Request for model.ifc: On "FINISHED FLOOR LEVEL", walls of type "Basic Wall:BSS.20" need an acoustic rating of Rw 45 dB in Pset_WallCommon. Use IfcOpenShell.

First a look at what the model holds.

```python
import ifcopenshell
import ifcopenshell.util.element

model = ifcopenshell.open("model.ifc")
print(model.schema)
storey = next(s for s in model.by_type("IfcBuildingStorey") if s.Name == "FINISHED FLOOR LEVEL")
walls = [e for e in ifcopenshell.util.element.get_decomposition(storey) if e.is_a("IfcWall")]
seen = {}
for e in walls:
    element_type = ifcopenshell.util.element.get_type(e)
    key = (element_type.Name if element_type != e and element_type else None, ifcopenshell.util.element.get_pset(e, "Pset_WallCommon", "AcousticRating"))
    seen[key] = seen.get(key, 0) + 1
for (name, value), count in sorted(seen.items(), key=str):
    print(count, "x", name, "|", value)
```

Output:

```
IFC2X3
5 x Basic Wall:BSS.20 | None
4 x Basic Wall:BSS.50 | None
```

```python
import ifcopenshell
import ifcopenshell.api.pset
import ifcopenshell.util.element

model = ifcopenshell.open("model.ifc")

storey = next(s for s in model.by_type("IfcBuildingStorey") if s.Name == "FINISHED FLOOR LEVEL")
walls = [e for e in ifcopenshell.util.element.get_decomposition(storey) if e.is_a("IfcWall")]

count = 0
for e in walls:
    element_type = ifcopenshell.util.element.get_type(e)
    if element_type in (None, e) or element_type.Name != "Basic Wall:BSS.20":
        continue
    # add_pset returns the element's existing set when there is one.
    pset = ifcopenshell.api.pset.add_pset(model, product=e, name="Pset_WallCommon")
    ifcopenshell.api.pset.edit_pset(model, pset=pset, properties={"AcousticRating": "Rw 45 dB"})
    count += 1

print(count, "walls updated")

model.write("model_rev.ifc")
```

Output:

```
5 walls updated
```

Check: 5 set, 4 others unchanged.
